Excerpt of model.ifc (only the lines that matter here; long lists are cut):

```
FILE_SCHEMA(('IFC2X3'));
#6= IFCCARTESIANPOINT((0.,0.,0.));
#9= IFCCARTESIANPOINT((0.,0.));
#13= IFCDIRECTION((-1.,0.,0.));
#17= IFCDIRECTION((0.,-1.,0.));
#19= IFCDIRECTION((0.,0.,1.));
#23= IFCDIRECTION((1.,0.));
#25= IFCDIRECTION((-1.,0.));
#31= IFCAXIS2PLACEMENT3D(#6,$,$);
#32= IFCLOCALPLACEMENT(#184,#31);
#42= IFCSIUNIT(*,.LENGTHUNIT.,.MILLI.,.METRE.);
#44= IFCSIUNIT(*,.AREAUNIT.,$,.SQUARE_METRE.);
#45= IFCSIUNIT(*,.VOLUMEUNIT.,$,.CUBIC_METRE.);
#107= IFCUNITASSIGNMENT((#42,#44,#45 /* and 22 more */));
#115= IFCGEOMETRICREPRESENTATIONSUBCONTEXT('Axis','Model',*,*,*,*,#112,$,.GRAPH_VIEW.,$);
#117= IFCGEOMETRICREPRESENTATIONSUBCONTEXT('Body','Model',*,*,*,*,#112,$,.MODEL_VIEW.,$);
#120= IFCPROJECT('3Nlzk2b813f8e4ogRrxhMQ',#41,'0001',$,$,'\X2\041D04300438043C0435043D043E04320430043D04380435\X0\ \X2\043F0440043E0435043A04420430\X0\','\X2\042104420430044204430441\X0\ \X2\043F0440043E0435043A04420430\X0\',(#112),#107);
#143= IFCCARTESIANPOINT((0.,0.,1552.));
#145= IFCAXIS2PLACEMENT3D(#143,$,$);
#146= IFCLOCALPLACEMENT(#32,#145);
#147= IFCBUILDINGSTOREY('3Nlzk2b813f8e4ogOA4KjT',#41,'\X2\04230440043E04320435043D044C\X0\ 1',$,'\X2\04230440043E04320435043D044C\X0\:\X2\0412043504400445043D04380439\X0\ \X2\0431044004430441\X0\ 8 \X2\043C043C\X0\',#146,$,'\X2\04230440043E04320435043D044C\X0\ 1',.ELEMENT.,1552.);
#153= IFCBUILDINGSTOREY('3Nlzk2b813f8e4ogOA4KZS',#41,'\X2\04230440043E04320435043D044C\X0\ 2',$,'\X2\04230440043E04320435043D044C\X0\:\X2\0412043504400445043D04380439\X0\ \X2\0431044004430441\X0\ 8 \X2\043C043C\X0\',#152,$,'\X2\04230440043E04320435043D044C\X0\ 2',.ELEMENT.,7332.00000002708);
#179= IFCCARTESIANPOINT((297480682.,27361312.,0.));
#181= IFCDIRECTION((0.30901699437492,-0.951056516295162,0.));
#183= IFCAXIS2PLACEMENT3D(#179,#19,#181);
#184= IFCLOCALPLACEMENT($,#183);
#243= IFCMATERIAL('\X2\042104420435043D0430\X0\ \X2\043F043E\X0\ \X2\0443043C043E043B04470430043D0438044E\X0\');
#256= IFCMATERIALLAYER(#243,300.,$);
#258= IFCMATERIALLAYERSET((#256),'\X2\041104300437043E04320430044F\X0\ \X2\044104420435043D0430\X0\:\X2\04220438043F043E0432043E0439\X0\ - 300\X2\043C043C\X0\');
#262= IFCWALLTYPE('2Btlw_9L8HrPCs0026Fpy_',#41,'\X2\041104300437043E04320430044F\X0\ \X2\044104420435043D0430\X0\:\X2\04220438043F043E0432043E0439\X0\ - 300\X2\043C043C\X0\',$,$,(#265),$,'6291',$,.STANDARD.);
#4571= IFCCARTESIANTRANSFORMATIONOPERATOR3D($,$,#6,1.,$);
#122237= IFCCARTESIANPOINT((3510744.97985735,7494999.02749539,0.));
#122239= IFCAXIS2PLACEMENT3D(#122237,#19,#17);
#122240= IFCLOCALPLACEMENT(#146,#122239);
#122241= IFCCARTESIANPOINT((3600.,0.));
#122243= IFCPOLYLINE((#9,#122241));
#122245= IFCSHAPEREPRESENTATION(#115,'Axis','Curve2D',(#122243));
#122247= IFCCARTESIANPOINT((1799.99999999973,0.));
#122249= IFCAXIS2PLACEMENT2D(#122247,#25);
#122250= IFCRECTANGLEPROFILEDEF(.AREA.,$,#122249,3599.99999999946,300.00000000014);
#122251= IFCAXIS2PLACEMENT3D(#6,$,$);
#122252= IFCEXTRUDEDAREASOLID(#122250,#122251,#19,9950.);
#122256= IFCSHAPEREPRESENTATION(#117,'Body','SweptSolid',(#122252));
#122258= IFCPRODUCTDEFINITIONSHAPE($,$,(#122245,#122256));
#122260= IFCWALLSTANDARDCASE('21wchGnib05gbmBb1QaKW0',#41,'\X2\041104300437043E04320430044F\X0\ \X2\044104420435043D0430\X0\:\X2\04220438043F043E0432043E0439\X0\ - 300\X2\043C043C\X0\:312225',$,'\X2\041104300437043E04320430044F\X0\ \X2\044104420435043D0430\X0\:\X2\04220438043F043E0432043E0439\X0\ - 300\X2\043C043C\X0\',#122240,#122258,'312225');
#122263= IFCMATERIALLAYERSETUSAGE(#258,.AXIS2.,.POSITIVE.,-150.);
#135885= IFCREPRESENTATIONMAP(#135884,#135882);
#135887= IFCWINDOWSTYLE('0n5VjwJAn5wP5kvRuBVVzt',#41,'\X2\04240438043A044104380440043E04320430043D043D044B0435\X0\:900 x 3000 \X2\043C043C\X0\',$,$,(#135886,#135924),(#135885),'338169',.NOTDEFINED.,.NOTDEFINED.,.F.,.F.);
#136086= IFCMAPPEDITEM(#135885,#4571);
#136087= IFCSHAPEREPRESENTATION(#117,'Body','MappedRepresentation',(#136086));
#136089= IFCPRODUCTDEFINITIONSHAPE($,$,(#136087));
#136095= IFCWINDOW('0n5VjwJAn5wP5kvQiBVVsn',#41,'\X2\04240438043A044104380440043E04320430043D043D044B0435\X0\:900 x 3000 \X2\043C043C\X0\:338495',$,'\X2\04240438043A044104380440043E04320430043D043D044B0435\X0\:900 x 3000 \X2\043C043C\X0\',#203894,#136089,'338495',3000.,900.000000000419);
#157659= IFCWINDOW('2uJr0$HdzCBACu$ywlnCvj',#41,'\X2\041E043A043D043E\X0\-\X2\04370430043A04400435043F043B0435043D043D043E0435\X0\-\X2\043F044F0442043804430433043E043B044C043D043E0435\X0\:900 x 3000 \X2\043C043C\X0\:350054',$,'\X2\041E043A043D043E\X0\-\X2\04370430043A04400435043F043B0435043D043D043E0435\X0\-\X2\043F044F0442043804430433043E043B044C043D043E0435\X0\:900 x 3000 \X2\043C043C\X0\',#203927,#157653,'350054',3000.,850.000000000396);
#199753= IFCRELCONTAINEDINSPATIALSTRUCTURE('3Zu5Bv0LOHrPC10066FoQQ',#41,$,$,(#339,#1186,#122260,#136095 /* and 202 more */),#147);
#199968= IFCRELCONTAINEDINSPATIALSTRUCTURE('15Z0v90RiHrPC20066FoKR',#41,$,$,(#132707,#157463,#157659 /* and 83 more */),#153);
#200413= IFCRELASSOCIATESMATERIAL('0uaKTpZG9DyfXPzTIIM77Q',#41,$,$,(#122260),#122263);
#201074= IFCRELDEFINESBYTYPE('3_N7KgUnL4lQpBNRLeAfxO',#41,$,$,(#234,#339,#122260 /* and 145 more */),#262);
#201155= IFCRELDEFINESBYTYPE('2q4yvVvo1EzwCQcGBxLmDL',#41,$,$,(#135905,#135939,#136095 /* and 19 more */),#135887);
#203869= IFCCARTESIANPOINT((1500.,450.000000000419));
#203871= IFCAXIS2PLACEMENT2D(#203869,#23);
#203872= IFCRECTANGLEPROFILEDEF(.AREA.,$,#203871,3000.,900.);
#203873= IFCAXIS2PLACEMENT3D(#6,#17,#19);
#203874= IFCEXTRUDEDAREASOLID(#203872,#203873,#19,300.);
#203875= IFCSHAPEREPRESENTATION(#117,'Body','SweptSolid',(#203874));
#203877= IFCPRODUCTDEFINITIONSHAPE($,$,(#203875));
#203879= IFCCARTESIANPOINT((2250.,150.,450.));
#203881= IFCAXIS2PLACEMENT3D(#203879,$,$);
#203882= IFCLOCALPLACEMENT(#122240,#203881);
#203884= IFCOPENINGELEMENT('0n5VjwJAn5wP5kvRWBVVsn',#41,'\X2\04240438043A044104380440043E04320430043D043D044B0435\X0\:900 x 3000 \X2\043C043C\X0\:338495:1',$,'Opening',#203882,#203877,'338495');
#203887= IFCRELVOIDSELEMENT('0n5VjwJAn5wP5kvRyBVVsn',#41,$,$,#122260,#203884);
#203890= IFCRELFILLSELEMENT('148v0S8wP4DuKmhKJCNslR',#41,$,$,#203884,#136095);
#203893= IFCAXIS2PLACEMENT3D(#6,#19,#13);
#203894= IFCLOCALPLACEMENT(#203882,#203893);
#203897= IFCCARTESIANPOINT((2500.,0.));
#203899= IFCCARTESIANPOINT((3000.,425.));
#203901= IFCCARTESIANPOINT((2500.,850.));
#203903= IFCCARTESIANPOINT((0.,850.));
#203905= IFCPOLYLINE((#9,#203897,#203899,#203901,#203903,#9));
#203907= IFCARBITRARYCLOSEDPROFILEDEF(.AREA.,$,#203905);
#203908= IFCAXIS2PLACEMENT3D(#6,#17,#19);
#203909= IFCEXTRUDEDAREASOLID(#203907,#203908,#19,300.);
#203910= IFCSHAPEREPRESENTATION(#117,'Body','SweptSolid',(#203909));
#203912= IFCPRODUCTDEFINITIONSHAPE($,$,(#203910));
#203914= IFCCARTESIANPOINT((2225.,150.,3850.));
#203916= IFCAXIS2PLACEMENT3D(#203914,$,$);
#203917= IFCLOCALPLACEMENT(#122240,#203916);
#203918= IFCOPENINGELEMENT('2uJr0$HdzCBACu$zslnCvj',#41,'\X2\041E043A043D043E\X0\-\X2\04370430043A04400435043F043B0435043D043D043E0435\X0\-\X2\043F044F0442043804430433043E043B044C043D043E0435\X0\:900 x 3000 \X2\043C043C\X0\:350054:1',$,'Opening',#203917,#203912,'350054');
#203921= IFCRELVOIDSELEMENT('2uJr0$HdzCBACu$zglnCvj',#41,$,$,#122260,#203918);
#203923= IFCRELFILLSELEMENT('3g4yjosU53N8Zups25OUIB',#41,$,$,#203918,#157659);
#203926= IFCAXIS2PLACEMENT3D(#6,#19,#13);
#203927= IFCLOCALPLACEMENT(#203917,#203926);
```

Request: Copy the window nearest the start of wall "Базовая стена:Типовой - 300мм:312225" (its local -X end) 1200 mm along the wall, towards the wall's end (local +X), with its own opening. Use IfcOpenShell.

```python
import ifcopenshell
import ifcopenshell.api.feature
import ifcopenshell.api.geometry
import ifcopenshell.api.root
import ifcopenshell.geom
import ifcopenshell.util.element
import ifcopenshell.util.placement
import ifcopenshell.util.shape
import ifcopenshell.util.unit

model = ifcopenshell.open("model.ifc")
unit_scale = ifcopenshell.util.unit.calculate_unit_scale(model)
settings = ifcopenshell.geom.settings()


def volume(element):
    """Net volume in cubic metres, openings subtracted."""
    shape = ifcopenshell.geom.create_shape(settings, element)
    return ifcopenshell.util.shape.get_volume(shape.geometry)


def reuse_history(source, copy):
    """copy_class also copies each property set's owner history, people and application; keep the originals."""
    for rel in copy.IsDefinedBy:
        if rel.is_a("IfcRelDefinesByProperties") and (history := rel.RelatingPropertyDefinition.OwnerHistory):
            rel.RelatingPropertyDefinition.OwnerHistory = source.OwnerHistory
            ifcopenshell.util.element.remove_deep2(model, history)


window = model.by_guid("0n5VjwJAn5wP5kvQiBVVsn")
opening = window.FillsVoids[0].RelatingOpeningElement
wall = opening.VoidsElements[0].RelatingBuildingElement
before = volume(wall)
shift = ifcopenshell.util.placement.get_local_placement(wall.ObjectPlacement)[:3, 0] * 1.2 / unit_scale

# copy_class copies the void relationship, type, container and properties, but no geometry.
new_opening = ifcopenshell.api.root.copy_class(model, product=opening)
new_opening.Representation = ifcopenshell.util.element.copy_deep(
    model, opening.Representation, exclude=["IfcGeometricRepresentationContext", "IfcRepresentationMap"]
)
new_opening.Name = "Фиксированные:900 x 3000 мм"
new_opening.Tag = None
new_window = ifcopenshell.api.root.copy_class(model, product=window)
new_window.Representation = ifcopenshell.util.element.copy_deep(
    model, window.Representation, exclude=["IfcGeometricRepresentationContext", "IfcRepresentationMap"]
)
new_window.Name = "Фиксированные:900 x 3000 мм"
new_window.Tag = None
reuse_history(window, new_window)
fills = ifcopenshell.api.feature.add_filling(model, opening=new_opening, element=new_window)
fills.OwnerHistory = new_window.OwnerHistory  # required in IFC2X3

for old, new in ((opening, new_opening), (window, new_window)):
    matrix = ifcopenshell.util.placement.get_local_placement(old.ObjectPlacement)
    matrix[:3, 3] += shift
    ifcopenshell.api.geometry.edit_object_placement(model, product=new, matrix=matrix, is_si=False)

after = volume(wall)

print(f"wall volume {before:.3f} -> {after:.3f} m3")

model.write("model_rev.ifc")
```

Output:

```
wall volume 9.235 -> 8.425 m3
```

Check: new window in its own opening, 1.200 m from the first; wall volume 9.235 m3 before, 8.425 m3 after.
